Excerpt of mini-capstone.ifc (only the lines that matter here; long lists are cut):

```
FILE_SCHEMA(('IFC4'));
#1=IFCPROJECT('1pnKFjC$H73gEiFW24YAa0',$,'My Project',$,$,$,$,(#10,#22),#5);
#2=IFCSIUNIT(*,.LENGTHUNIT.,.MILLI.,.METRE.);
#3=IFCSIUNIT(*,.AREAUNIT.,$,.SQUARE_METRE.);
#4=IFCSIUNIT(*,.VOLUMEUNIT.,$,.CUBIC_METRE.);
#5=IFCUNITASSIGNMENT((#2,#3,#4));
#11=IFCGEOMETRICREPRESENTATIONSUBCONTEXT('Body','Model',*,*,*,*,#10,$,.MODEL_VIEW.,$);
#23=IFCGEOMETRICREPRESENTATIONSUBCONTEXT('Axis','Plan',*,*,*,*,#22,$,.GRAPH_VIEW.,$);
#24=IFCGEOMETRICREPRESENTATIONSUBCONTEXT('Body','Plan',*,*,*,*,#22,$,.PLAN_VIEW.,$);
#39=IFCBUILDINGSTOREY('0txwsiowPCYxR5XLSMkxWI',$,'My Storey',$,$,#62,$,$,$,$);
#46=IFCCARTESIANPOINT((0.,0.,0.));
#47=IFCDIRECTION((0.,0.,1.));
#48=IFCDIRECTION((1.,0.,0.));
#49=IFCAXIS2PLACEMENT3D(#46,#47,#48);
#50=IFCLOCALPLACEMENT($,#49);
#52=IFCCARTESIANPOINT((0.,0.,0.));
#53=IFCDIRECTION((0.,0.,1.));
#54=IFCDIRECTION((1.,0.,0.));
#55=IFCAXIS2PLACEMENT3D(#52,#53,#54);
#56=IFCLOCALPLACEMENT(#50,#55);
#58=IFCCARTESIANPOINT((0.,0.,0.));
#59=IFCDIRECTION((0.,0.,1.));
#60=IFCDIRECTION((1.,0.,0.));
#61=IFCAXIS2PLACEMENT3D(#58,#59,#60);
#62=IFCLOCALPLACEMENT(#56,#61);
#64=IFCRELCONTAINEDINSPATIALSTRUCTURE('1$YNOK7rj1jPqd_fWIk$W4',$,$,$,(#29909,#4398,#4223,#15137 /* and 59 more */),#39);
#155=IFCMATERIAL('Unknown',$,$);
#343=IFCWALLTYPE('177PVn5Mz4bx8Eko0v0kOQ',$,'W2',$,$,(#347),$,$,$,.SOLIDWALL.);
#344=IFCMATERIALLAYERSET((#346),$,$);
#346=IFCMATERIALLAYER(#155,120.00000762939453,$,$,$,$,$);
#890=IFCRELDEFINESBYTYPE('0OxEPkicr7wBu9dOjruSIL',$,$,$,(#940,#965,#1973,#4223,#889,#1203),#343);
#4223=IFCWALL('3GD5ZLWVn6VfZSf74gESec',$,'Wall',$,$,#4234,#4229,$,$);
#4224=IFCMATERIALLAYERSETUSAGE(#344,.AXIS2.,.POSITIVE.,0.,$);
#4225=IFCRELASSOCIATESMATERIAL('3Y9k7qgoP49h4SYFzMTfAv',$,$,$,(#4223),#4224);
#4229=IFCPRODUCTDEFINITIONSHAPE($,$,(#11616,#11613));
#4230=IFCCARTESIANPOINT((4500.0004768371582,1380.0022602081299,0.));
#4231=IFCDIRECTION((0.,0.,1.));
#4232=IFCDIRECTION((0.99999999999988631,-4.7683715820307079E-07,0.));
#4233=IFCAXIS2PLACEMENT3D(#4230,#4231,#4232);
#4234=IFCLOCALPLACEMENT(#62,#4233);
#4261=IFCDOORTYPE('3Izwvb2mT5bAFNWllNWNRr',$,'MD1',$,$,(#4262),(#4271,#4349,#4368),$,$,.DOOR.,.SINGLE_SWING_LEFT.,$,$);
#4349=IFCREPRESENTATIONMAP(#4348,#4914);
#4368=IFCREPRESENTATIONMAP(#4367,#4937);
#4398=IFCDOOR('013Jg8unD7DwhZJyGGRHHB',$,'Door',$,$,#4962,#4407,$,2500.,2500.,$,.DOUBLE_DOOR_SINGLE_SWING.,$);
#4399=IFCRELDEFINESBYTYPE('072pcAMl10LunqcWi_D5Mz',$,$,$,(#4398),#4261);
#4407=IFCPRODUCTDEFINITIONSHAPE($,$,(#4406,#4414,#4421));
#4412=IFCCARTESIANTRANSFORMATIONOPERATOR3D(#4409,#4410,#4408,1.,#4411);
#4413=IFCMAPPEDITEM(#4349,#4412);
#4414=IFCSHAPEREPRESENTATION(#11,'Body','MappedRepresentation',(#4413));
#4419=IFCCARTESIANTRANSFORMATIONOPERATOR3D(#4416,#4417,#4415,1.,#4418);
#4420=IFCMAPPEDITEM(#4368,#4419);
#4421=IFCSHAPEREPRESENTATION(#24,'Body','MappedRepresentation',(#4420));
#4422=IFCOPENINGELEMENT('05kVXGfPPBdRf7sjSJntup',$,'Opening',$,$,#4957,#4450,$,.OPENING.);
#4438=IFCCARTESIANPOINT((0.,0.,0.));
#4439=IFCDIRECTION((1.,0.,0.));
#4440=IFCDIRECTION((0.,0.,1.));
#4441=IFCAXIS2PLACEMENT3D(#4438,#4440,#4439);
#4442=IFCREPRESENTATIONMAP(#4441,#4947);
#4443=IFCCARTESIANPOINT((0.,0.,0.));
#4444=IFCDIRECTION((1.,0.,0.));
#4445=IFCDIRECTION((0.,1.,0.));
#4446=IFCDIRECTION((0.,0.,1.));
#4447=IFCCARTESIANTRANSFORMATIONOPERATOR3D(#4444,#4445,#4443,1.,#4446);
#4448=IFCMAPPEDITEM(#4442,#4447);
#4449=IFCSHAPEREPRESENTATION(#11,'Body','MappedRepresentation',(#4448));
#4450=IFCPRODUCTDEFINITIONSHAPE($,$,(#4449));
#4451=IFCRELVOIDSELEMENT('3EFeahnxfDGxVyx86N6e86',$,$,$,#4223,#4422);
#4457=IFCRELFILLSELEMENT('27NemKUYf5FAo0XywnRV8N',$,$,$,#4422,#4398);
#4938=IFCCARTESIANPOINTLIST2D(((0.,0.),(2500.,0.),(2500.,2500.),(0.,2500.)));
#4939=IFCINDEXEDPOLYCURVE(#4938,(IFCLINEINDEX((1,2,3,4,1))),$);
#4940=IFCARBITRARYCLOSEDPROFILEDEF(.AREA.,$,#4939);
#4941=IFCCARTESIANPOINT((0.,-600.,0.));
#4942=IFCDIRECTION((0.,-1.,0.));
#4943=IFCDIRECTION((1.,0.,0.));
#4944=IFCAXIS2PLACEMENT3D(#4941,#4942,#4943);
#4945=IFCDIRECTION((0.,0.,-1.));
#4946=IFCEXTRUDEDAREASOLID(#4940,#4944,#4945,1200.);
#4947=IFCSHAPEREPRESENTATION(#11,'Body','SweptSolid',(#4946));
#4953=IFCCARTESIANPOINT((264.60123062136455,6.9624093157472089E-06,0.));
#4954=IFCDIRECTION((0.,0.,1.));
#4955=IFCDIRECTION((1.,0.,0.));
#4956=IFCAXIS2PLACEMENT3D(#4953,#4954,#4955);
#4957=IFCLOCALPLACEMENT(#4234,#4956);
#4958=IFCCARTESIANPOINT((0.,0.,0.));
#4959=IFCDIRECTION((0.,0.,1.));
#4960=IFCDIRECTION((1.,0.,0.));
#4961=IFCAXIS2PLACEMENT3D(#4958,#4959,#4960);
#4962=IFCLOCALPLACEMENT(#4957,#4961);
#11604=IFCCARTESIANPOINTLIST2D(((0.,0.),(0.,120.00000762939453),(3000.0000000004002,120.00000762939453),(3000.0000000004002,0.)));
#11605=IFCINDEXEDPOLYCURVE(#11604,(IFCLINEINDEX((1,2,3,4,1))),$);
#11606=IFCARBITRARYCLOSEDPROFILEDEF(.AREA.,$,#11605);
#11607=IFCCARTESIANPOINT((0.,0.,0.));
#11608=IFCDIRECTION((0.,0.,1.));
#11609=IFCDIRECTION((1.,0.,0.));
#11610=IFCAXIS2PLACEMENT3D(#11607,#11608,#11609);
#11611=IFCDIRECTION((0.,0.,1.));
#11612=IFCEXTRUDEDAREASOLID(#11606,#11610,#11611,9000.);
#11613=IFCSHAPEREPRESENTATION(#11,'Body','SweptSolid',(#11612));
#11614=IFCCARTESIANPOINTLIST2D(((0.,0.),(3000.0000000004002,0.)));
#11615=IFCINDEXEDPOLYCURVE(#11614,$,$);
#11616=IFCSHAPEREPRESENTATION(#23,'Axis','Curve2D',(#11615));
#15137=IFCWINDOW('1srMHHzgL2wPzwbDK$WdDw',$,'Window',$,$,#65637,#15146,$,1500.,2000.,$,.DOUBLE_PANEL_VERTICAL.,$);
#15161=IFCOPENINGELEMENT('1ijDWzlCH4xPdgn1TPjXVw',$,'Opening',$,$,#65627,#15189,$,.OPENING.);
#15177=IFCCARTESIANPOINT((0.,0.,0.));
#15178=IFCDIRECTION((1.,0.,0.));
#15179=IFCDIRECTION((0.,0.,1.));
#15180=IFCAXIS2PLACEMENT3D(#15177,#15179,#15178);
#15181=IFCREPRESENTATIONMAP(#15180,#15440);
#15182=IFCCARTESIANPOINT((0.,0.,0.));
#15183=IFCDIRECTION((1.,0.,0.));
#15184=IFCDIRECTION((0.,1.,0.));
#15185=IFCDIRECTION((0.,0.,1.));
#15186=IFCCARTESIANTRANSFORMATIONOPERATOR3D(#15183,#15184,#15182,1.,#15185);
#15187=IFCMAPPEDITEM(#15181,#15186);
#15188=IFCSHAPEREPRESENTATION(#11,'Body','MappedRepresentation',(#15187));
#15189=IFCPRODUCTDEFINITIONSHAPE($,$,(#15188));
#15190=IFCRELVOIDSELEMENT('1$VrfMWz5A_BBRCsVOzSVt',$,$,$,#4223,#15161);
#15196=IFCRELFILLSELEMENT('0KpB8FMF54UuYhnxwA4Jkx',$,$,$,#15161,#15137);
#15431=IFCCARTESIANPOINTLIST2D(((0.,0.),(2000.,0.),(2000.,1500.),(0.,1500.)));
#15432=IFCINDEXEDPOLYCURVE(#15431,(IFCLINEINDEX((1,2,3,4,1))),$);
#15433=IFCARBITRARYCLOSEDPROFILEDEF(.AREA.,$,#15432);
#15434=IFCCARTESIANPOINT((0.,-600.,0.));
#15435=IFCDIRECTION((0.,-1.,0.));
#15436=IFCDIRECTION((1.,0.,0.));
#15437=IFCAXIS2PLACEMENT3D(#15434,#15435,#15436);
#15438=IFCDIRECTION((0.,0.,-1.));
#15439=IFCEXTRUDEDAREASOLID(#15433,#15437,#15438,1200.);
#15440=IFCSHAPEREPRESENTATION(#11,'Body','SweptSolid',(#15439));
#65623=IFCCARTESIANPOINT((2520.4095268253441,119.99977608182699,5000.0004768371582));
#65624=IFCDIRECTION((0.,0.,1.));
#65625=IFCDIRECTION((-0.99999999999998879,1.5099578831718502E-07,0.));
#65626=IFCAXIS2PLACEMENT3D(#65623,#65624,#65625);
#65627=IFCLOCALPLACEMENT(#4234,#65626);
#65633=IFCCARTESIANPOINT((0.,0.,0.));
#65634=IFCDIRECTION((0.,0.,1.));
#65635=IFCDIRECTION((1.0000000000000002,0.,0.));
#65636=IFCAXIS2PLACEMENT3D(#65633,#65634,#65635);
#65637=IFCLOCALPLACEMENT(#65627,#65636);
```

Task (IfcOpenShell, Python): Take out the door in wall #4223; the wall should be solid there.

```python
import ifcopenshell
import ifcopenshell.api.feature
import ifcopenshell.api.root
import ifcopenshell.geom
import ifcopenshell.util.shape

model = ifcopenshell.open("mini-capstone.ifc")
settings = ifcopenshell.geom.settings()


def volume(element):
    """Net volume in cubic metres, openings subtracted."""
    shape = ifcopenshell.geom.create_shape(settings, element)
    return ifcopenshell.util.shape.get_volume(shape.geometry)


door = model.by_id(4398)
opening = door.FillsVoids[0].RelatingOpeningElement
wall = opening.VoidsElements[0].RelatingBuildingElement
before = volume(wall)

ifcopenshell.api.root.remove_product(model, product=door)
ifcopenshell.api.feature.remove_feature(model, feature=opening)

after = volume(wall)

print(f"wall volume {before:.3f} -> {after:.3f} m3")

model.write("mini-capstone_rev.ifc")
```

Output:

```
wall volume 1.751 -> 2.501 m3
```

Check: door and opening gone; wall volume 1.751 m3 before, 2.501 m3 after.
